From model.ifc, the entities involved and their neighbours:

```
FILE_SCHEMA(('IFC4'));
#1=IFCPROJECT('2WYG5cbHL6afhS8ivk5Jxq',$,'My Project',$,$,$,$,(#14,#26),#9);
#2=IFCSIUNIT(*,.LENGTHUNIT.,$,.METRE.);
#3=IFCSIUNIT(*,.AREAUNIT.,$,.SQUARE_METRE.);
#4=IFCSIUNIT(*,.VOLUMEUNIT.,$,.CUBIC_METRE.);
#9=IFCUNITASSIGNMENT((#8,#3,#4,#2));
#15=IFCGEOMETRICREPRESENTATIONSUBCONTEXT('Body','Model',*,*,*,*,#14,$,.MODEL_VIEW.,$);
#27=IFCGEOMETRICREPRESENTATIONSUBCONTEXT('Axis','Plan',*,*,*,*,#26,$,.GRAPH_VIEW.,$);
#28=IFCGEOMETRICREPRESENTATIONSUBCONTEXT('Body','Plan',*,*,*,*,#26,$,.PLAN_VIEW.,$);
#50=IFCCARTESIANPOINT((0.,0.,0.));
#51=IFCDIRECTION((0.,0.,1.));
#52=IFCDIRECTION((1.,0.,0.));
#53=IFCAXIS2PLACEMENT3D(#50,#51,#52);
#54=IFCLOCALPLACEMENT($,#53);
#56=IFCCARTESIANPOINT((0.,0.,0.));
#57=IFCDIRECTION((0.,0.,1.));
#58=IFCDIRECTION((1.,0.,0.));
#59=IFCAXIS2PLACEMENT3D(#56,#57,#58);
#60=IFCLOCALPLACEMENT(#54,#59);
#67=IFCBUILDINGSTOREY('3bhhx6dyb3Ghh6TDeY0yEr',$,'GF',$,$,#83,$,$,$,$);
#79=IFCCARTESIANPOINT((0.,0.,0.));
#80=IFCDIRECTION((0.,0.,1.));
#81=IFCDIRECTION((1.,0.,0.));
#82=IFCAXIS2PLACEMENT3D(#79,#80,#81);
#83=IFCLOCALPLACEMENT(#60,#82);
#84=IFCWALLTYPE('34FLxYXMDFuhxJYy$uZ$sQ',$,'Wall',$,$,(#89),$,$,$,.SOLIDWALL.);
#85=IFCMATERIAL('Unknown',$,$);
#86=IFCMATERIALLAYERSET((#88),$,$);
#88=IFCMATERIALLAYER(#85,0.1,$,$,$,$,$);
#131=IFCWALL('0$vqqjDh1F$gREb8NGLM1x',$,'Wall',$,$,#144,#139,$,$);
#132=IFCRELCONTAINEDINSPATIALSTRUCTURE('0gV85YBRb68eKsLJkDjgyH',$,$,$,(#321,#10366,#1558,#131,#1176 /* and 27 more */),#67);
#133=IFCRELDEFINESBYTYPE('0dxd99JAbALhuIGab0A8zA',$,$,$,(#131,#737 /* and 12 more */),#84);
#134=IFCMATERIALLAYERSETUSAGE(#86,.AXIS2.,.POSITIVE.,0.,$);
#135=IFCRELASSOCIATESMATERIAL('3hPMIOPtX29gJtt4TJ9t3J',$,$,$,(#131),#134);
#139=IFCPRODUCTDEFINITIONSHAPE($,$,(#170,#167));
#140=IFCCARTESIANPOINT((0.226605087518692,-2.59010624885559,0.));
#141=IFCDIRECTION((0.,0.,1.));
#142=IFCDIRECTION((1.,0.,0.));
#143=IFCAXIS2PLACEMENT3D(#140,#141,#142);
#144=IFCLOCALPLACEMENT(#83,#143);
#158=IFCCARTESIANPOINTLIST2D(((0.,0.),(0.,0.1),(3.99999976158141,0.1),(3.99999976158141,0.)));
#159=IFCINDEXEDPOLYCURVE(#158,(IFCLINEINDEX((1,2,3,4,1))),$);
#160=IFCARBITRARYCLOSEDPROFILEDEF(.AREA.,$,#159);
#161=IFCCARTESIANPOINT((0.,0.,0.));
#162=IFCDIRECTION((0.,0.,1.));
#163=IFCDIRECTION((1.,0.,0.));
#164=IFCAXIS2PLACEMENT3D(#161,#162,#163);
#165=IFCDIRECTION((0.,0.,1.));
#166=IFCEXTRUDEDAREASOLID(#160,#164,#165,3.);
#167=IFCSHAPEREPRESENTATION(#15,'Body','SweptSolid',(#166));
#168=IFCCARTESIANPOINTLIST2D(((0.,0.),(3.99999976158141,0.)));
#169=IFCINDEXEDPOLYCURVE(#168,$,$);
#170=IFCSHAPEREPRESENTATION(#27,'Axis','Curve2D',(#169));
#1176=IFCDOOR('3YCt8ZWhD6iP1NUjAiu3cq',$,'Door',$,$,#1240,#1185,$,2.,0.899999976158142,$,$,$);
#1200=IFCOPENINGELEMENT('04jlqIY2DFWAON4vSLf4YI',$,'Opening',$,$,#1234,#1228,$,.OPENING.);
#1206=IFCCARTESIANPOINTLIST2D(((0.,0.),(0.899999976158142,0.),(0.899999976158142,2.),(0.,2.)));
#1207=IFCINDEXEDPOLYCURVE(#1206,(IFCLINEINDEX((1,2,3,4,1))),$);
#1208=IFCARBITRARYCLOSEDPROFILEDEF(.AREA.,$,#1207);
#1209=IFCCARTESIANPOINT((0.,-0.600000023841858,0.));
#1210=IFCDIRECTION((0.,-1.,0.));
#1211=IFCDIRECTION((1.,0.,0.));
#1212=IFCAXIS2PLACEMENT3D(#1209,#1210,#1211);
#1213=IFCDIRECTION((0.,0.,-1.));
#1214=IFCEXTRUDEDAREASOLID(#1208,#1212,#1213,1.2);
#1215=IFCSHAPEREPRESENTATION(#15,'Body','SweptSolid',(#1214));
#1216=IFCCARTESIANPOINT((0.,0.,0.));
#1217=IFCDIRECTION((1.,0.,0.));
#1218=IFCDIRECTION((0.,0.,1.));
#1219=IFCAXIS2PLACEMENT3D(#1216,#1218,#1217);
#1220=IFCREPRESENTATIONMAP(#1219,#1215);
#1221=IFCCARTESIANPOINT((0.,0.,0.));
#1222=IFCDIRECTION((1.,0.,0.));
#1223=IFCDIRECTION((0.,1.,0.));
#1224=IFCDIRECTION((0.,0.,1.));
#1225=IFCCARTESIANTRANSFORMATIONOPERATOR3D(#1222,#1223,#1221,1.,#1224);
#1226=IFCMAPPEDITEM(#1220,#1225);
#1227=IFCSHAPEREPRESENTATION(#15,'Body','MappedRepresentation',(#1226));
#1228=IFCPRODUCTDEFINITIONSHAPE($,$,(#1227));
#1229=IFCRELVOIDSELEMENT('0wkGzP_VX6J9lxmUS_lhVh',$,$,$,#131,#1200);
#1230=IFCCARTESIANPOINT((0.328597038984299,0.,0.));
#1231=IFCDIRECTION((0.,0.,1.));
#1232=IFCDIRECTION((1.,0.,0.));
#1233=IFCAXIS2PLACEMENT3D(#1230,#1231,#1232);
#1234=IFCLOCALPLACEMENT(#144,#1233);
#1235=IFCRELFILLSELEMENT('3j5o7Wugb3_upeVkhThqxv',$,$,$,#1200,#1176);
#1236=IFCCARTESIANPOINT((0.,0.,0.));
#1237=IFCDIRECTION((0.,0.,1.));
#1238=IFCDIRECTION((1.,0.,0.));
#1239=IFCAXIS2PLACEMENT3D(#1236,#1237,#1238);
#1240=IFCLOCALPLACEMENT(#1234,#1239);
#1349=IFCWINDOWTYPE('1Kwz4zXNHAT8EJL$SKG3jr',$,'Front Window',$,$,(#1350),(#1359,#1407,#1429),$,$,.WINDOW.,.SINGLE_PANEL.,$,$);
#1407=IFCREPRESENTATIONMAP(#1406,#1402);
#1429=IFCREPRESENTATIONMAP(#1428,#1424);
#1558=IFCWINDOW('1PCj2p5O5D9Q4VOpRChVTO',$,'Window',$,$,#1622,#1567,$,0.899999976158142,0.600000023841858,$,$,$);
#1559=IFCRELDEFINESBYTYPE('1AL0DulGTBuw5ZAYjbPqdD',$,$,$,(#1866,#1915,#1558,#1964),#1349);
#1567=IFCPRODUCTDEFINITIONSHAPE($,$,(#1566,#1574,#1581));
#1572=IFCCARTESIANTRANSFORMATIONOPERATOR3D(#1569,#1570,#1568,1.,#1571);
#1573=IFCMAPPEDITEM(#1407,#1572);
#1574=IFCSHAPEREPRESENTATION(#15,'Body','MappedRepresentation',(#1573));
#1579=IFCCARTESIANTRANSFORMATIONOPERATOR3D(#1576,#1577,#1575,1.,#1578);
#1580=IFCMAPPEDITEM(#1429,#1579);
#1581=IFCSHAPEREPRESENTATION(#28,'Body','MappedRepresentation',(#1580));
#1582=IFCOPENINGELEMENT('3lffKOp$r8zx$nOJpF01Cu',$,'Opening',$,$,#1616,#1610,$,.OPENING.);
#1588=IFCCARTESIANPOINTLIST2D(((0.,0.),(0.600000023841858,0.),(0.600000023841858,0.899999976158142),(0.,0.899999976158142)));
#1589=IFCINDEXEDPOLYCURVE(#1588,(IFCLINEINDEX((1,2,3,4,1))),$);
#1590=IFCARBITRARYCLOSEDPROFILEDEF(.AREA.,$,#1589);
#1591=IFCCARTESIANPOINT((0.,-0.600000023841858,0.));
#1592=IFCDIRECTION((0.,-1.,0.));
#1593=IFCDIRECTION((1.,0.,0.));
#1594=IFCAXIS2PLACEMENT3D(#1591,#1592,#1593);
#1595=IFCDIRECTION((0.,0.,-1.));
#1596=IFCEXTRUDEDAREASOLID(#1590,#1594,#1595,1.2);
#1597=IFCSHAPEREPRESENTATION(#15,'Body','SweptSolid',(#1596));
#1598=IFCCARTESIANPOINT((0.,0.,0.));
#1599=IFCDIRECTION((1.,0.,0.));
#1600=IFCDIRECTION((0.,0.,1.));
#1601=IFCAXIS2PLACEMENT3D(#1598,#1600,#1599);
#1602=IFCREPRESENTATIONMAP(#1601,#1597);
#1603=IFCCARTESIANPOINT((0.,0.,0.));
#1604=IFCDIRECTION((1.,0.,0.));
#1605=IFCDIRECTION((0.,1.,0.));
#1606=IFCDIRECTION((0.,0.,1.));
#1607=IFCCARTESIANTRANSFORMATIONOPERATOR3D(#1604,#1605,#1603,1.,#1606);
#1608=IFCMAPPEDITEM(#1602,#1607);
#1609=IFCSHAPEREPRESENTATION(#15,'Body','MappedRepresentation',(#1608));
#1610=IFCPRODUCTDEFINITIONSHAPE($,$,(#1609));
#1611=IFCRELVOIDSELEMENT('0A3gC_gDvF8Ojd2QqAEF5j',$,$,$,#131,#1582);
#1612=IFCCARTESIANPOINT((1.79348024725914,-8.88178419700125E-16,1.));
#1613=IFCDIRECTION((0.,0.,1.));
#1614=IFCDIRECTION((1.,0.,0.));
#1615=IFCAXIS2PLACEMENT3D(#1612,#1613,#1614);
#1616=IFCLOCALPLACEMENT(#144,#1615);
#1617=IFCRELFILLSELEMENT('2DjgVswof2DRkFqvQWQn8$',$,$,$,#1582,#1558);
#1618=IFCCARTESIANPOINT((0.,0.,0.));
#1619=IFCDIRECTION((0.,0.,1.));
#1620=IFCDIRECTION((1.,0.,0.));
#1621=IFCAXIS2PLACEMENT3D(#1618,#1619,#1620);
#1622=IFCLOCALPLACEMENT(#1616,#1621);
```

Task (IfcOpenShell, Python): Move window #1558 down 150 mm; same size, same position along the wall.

```python
import numpy as np
import ifcopenshell
import ifcopenshell.api.geometry
import ifcopenshell.util.placement
import ifcopenshell.util.unit

model = ifcopenshell.open("model.ifc")
unit_scale = ifcopenshell.util.unit.calculate_unit_scale(model)

window = model.by_id(1558)
opening = window.FillsVoids[0].RelatingOpeningElement
dz = -0.15 / unit_scale

shift = np.array([0.0, 0.0, dz])
# The window is placed relative to its opening, so it follows when the opening moves.
matrix = ifcopenshell.util.placement.get_local_placement(opening.ObjectPlacement)
matrix[:3, 3] += shift
ifcopenshell.api.geometry.edit_object_placement(
    model, product=opening, matrix=matrix, is_si=False, should_transform_children=True
)

print(f"moved by {dz * unit_scale:+.3f} m")

model.write("model_rev.ifc")
```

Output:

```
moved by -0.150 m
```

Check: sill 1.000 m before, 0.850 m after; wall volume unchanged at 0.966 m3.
